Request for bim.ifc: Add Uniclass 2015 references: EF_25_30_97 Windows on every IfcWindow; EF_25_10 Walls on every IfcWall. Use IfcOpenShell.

First a look at what the model holds.

```python
import ifcopenshell

model = ifcopenshell.open("bim.ifc")
print(model.schema)
print("classifications:", [c.Name for c in model.by_type("IfcClassification")])
for ifc_class in ("IfcDoor", "IfcRoof", "IfcStair", "IfcWall", "IfcWindow"):
    print(ifc_class, len(model.by_type(ifc_class)))
```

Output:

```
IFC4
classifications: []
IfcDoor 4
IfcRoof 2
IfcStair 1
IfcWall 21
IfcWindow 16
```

```python
import ifcopenshell
import ifcopenshell.api.classification

model = ifcopenshell.open("bim.ifc")

system = ifcopenshell.api.classification.add_classification(model, classification="Uniclass 2015")

codes = {
    "IfcWindow": ("EF_25_30_97", "Windows"),
    "IfcWall": ("EF_25_10", "Walls"),
}
for ifc_class, (code, name) in codes.items():
    products = model.by_type(ifc_class)
    ifcopenshell.api.classification.add_reference(
        model, products=products, classification=system, identification=code, name=name
    )
    print(code, len(products))

model.write("bim-out.ifc")
```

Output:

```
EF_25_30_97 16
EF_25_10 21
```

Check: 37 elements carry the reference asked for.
